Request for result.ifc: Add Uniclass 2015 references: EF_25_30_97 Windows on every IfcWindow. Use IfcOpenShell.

First a look at what the model holds.

```python
import ifcopenshell

model = ifcopenshell.open("result.ifc")
print(model.schema)
print("classifications:", [c.Name for c in model.by_type("IfcClassification")])
for ifc_class in ("IfcDoor", "IfcRoof", "IfcStair", "IfcWall", "IfcWindow"):
    print(ifc_class, len(model.by_type(ifc_class)))
```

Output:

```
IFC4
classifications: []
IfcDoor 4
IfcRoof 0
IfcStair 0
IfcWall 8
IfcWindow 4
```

```python
import ifcopenshell
import ifcopenshell.api.classification

model = ifcopenshell.open("result.ifc")

system = ifcopenshell.api.classification.add_classification(model, classification="Uniclass 2015")

codes = {
    "IfcWindow": ("EF_25_30_97", "Windows"),
}
for ifc_class, (code, name) in codes.items():
    products = model.by_type(ifc_class)
    ifcopenshell.api.classification.add_reference(
        model, products=products, classification=system, identification=code, name=name
    )
    print(code, len(products))

model.write("result_v2.ifc")
```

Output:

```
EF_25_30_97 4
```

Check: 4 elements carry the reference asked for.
